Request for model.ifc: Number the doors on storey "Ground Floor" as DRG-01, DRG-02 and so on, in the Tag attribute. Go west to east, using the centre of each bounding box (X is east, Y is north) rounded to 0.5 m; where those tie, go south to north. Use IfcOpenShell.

First a look at what the model holds.

```python
import ifcopenshell
import ifcopenshell.util.element
import ifcopenshell.util.placement

model = ifcopenshell.open("model.ifc")
print(model.schema)
storey = next(s for s in model.by_type("IfcBuildingStorey") if s.Name == "Ground Floor")
doors = [e for e in ifcopenshell.util.element.get_decomposition(storey) if e.is_a("IfcDoor")]
for e in sorted(doors, key=lambda e: e.id()):
    origin = ifcopenshell.util.placement.get_local_placement(e.ObjectPlacement)[:3, 3]
    print(e.id(), e.Tag, e.Name, origin.round(2) + 0.0, sep=" | ")
```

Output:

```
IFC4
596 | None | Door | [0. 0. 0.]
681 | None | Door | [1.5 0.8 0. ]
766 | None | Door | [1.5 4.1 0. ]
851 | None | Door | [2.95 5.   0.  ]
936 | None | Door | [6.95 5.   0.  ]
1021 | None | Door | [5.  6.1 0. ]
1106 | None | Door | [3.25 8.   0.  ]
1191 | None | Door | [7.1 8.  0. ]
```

```python
import ifcopenshell
import ifcopenshell.geom
import ifcopenshell.util.element
import ifcopenshell.util.shape

model = ifcopenshell.open("model.ifc")
settings = ifcopenshell.geom.settings()
settings.set("use-world-coords", True)


def centre(element):
    shape = ifcopenshell.geom.create_shape(settings, element)
    return ifcopenshell.util.shape.get_bbox_centroid(shape.geometry)


storey = next(s for s in model.by_type("IfcBuildingStorey") if s.Name == "Ground Floor")
doors = [e for e in ifcopenshell.util.element.get_decomposition(storey) if e.is_a("IfcDoor")]

# Insertion points can sit at a corner or the storey origin, so sort by the geometry (in metres).
centres = {e: centre(e) for e in doors}
doors.sort(key=lambda e: (round(centres[e][0] / 0.5), centres[e][1]))

for i, e in enumerate(doors, start=1):
    number = f"DRG-{i:02d}"
    e.Tag = number
    print(e.id(), number)

model.write("model-out.ifc")
```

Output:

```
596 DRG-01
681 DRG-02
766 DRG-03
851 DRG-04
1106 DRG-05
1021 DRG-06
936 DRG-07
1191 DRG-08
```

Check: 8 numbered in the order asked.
